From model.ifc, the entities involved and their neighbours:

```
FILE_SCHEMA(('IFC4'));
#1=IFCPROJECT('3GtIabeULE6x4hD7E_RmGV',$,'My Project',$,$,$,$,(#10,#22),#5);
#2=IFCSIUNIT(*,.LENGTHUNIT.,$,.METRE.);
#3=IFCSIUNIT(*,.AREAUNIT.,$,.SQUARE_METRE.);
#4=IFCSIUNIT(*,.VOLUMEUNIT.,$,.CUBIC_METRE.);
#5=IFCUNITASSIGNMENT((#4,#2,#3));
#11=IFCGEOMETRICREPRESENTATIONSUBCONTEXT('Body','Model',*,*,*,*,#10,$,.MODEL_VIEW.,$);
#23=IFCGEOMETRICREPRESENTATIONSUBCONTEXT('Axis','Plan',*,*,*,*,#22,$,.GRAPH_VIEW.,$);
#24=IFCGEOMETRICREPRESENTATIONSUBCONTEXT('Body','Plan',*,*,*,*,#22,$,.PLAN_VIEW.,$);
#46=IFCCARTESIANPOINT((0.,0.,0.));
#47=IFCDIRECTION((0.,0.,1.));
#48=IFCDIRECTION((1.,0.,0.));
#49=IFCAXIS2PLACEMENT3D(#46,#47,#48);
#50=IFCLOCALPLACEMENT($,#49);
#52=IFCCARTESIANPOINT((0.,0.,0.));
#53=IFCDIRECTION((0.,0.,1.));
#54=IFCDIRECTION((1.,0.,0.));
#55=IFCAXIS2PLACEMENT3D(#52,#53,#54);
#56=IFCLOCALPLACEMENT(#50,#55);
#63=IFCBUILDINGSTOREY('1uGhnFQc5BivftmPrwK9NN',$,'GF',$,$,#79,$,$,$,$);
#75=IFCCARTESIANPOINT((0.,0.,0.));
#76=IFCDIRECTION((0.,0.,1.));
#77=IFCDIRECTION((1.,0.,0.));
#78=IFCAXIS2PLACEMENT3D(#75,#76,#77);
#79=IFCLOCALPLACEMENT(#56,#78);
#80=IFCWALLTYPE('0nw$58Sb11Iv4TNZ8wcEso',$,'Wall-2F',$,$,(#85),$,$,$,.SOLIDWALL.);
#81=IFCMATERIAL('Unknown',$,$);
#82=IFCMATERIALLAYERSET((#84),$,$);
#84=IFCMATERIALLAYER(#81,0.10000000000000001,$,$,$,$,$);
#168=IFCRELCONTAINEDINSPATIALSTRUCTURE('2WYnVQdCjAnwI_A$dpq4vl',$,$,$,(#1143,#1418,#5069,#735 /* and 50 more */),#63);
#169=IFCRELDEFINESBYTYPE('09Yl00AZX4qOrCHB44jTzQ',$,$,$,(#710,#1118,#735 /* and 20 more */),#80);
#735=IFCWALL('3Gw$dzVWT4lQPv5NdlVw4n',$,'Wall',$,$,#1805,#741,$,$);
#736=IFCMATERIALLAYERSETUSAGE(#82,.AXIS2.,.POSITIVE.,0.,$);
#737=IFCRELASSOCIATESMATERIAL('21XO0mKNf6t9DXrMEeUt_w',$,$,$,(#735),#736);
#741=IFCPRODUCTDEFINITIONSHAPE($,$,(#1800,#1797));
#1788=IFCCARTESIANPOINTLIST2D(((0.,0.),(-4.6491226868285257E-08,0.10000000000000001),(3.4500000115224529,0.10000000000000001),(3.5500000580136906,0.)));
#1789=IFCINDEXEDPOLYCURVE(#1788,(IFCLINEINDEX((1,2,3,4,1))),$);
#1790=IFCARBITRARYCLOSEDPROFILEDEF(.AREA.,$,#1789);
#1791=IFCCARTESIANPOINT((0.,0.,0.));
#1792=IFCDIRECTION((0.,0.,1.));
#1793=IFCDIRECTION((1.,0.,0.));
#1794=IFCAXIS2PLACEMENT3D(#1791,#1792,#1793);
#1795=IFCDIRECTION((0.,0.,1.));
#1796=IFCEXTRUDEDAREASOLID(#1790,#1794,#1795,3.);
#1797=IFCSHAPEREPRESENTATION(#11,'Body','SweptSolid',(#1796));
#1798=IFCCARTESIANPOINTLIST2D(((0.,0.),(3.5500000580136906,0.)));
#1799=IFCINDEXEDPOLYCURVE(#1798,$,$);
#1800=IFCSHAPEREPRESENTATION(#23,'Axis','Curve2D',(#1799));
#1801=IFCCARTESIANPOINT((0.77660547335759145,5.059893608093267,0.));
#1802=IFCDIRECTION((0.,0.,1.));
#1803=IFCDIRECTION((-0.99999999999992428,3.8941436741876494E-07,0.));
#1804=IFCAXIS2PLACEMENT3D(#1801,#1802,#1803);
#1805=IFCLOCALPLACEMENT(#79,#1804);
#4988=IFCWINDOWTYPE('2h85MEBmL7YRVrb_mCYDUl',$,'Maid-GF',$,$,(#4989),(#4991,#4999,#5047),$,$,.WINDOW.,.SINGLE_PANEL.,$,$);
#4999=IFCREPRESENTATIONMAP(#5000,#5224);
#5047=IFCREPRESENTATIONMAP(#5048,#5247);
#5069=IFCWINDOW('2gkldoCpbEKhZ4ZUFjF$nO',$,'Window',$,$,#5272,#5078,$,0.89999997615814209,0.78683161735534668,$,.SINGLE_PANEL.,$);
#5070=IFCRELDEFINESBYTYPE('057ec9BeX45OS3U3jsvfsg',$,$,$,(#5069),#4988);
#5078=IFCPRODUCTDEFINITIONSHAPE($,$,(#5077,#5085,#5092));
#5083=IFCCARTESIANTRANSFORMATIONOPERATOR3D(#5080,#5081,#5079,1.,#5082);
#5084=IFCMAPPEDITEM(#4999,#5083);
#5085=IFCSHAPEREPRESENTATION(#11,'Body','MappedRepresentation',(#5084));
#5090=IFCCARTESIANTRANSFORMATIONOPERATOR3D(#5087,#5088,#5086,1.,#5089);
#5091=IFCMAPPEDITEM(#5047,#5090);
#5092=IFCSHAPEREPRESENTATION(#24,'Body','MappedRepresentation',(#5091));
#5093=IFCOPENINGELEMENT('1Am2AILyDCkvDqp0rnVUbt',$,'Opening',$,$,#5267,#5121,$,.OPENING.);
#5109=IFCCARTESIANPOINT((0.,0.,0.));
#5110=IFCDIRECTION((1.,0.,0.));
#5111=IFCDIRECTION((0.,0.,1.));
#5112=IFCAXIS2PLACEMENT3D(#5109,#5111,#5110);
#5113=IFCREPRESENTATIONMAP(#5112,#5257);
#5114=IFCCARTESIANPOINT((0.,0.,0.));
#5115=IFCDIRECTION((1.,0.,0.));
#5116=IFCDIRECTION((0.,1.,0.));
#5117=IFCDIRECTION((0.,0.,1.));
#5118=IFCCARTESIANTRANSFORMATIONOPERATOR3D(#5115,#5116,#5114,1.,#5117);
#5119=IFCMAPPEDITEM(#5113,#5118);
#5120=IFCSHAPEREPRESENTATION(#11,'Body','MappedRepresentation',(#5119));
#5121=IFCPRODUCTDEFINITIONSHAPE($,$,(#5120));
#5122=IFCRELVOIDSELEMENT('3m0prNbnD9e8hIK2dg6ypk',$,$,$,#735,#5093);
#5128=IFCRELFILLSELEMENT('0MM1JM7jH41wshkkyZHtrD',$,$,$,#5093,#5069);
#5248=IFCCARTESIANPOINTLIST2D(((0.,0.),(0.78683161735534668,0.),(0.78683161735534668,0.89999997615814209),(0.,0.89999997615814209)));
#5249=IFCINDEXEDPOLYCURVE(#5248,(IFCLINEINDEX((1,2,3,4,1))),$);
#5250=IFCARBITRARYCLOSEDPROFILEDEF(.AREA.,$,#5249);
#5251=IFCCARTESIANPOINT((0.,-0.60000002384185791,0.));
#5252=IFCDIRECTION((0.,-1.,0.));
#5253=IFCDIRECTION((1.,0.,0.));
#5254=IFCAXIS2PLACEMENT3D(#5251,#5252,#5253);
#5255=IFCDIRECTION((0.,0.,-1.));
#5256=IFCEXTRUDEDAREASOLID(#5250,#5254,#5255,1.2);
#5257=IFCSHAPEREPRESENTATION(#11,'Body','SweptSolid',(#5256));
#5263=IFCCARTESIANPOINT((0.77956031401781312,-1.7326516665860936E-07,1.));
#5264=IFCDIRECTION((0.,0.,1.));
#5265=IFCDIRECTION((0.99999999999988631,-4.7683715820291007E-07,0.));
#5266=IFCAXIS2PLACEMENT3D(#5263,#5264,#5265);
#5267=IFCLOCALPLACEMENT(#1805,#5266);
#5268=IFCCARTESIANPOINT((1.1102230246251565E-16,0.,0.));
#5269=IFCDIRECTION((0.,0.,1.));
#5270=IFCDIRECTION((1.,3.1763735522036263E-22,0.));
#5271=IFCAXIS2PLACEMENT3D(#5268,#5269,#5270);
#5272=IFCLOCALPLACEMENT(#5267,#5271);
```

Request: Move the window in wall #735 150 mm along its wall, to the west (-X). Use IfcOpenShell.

```python
import ifcopenshell
import ifcopenshell.api.geometry
import ifcopenshell.util.placement
import ifcopenshell.util.unit

model = ifcopenshell.open("model.ifc")
unit_scale = ifcopenshell.util.unit.calculate_unit_scale(model)

window = model.by_id(5069)
opening = window.FillsVoids[0].RelatingOpeningElement
wall = opening.VoidsElements[0].RelatingBuildingElement

wall_matrix = ifcopenshell.util.placement.get_local_placement(wall.ObjectPlacement)
shift = wall_matrix[:3, 0] * 0.15 / unit_scale
before = ifcopenshell.util.placement.get_local_placement(window.ObjectPlacement)[:3, 3].copy()

# The window is placed relative to its opening, so it follows when the opening moves.
matrix = ifcopenshell.util.placement.get_local_placement(opening.ObjectPlacement)
matrix[:3, 3] += shift
ifcopenshell.api.geometry.edit_object_placement(
    model, product=opening, matrix=matrix, is_si=False, should_transform_children=True
)

after = ifcopenshell.util.placement.get_local_placement(window.ObjectPlacement)[:3, 3]
print("window moved by", (after - before).round(3) + 0.0)

model.write("model_updated.ifc")
```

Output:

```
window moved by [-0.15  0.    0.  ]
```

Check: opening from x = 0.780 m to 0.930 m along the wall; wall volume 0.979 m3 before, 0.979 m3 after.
